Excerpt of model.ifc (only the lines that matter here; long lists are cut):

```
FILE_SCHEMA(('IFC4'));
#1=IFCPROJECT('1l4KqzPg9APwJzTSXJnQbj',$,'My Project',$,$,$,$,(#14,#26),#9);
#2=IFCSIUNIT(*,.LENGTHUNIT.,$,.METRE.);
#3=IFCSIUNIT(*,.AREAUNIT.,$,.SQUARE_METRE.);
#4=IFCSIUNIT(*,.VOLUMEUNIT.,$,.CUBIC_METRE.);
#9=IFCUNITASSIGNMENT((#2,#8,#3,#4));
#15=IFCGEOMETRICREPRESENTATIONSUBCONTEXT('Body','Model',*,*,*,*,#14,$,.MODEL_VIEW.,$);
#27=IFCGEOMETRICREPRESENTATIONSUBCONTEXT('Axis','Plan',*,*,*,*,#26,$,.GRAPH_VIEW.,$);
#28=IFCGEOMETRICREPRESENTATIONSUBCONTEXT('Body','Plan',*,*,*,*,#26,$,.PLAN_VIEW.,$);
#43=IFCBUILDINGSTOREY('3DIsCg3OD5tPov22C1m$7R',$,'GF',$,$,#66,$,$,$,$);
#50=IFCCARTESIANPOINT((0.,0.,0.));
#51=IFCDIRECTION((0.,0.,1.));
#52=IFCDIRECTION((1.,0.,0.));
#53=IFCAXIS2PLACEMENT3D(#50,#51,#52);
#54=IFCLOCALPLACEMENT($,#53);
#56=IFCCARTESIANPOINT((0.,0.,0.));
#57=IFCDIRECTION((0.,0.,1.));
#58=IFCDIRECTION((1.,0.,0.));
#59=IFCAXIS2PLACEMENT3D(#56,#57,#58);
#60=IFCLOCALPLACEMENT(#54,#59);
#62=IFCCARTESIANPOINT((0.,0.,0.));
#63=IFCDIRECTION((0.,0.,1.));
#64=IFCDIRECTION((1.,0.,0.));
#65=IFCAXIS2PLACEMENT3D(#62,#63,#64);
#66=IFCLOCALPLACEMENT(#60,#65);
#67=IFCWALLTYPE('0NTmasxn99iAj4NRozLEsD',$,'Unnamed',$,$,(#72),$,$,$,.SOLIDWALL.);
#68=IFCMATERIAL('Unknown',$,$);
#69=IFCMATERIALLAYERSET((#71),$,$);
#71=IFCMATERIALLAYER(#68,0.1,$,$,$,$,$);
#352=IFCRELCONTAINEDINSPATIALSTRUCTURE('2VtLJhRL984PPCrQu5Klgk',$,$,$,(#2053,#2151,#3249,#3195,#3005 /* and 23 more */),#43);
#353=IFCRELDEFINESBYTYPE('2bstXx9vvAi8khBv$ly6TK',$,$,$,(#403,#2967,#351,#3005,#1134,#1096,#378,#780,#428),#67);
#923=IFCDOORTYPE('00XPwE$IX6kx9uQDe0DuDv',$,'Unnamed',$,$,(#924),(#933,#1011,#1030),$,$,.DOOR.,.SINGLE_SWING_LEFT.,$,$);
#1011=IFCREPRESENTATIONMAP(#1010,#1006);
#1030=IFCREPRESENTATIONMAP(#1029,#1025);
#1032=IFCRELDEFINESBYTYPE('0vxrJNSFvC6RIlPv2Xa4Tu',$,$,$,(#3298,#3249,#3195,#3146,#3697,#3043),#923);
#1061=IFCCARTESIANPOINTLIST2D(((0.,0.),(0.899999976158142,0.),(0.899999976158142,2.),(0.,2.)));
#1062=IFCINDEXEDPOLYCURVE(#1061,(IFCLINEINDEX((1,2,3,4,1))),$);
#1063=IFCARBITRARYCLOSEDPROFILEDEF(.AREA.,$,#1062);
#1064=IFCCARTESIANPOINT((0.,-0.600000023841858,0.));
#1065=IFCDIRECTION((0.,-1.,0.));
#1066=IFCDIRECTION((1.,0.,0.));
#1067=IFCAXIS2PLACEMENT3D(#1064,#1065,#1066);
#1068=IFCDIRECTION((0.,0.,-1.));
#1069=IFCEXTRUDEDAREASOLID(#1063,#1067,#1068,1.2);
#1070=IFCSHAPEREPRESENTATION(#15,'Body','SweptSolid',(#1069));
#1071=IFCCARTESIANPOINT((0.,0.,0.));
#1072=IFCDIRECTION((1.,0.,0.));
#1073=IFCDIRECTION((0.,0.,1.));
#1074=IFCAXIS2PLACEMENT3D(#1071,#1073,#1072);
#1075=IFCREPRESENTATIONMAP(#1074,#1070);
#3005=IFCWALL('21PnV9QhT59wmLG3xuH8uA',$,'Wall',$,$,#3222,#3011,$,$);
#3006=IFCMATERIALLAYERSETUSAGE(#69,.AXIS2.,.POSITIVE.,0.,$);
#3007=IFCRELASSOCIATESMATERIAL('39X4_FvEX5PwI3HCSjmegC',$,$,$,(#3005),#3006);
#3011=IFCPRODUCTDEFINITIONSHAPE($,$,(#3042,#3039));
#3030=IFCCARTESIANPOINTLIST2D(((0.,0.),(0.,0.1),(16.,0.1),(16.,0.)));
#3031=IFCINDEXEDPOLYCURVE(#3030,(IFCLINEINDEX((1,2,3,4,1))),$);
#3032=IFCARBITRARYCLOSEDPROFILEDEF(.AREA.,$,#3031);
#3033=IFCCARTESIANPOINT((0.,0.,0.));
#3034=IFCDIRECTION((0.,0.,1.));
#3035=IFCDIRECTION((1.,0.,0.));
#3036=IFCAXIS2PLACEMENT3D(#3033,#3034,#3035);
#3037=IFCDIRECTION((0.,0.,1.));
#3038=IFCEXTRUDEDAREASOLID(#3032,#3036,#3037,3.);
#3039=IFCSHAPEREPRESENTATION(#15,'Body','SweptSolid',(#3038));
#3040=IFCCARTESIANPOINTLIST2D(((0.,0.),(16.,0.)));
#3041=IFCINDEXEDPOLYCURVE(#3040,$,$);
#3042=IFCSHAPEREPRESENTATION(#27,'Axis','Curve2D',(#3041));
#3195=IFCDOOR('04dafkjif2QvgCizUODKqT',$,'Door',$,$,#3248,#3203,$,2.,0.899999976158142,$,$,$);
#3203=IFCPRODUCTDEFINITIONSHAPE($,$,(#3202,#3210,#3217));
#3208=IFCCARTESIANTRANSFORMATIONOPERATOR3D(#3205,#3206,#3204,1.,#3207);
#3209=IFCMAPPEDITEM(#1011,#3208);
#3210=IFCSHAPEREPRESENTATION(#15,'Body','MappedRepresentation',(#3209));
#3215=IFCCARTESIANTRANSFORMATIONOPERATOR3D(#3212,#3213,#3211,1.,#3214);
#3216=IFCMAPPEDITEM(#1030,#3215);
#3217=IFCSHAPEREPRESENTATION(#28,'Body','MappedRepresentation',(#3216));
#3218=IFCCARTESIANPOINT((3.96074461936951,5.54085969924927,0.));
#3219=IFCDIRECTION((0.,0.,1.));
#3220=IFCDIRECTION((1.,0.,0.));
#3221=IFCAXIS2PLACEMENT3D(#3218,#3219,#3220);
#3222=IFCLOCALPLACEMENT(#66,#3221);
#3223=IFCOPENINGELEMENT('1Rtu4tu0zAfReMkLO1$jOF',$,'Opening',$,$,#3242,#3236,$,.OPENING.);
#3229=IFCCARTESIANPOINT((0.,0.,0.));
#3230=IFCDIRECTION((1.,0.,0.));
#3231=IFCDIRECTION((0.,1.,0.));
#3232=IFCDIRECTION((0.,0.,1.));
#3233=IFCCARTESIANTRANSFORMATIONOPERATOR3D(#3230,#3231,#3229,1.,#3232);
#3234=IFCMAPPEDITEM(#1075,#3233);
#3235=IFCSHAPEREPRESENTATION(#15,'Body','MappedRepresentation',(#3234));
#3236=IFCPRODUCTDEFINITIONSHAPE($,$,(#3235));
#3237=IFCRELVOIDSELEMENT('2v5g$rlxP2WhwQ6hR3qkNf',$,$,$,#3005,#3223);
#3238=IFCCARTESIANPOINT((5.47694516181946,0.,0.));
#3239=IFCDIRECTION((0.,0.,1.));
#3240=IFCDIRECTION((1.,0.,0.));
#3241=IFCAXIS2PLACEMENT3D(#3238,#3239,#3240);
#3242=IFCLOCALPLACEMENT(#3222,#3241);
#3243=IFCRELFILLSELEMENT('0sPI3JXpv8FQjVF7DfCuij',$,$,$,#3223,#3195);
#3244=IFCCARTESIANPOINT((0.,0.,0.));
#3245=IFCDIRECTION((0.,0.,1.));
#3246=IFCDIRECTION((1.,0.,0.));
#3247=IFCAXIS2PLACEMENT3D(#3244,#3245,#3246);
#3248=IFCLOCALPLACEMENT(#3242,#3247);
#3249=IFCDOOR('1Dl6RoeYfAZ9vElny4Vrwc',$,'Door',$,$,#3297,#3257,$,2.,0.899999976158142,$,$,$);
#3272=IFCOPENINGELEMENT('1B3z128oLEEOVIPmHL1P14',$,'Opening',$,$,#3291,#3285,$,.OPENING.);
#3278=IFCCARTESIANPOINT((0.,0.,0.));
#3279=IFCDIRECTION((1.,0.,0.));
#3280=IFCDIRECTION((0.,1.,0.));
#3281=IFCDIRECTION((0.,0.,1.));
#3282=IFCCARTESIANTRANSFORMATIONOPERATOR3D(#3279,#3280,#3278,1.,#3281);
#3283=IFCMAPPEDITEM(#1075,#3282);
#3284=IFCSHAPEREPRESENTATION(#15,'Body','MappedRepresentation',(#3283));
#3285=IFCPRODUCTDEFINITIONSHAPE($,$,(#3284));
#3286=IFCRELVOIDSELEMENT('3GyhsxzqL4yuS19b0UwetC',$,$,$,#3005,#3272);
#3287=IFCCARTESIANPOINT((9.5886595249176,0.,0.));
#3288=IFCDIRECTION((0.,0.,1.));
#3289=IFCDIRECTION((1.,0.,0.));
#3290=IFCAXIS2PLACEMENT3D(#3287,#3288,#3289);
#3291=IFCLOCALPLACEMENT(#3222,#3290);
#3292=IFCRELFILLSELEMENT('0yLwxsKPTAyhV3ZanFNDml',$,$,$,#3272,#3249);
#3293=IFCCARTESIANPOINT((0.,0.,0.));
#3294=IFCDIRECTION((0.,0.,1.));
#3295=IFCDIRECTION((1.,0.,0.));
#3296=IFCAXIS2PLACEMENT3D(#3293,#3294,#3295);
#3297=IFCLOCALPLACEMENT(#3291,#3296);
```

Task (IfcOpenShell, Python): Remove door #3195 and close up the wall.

```python
import ifcopenshell
import ifcopenshell.api.feature
import ifcopenshell.api.root
import ifcopenshell.geom
import ifcopenshell.util.shape

model = ifcopenshell.open("model.ifc")
settings = ifcopenshell.geom.settings()


def volume(element):
    """Net volume in cubic metres, openings subtracted."""
    shape = ifcopenshell.geom.create_shape(settings, element)
    return ifcopenshell.util.shape.get_volume(shape.geometry)


door = model.by_id(3195)
opening = door.FillsVoids[0].RelatingOpeningElement
wall = opening.VoidsElements[0].RelatingBuildingElement
before = volume(wall)

ifcopenshell.api.root.remove_product(model, product=door)
ifcopenshell.api.feature.remove_feature(model, feature=opening)

after = volume(wall)

print(f"wall volume {before:.3f} -> {after:.3f} m3")

model.write("model_v2.ifc")
```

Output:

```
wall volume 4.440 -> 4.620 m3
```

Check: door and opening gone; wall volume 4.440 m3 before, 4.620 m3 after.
